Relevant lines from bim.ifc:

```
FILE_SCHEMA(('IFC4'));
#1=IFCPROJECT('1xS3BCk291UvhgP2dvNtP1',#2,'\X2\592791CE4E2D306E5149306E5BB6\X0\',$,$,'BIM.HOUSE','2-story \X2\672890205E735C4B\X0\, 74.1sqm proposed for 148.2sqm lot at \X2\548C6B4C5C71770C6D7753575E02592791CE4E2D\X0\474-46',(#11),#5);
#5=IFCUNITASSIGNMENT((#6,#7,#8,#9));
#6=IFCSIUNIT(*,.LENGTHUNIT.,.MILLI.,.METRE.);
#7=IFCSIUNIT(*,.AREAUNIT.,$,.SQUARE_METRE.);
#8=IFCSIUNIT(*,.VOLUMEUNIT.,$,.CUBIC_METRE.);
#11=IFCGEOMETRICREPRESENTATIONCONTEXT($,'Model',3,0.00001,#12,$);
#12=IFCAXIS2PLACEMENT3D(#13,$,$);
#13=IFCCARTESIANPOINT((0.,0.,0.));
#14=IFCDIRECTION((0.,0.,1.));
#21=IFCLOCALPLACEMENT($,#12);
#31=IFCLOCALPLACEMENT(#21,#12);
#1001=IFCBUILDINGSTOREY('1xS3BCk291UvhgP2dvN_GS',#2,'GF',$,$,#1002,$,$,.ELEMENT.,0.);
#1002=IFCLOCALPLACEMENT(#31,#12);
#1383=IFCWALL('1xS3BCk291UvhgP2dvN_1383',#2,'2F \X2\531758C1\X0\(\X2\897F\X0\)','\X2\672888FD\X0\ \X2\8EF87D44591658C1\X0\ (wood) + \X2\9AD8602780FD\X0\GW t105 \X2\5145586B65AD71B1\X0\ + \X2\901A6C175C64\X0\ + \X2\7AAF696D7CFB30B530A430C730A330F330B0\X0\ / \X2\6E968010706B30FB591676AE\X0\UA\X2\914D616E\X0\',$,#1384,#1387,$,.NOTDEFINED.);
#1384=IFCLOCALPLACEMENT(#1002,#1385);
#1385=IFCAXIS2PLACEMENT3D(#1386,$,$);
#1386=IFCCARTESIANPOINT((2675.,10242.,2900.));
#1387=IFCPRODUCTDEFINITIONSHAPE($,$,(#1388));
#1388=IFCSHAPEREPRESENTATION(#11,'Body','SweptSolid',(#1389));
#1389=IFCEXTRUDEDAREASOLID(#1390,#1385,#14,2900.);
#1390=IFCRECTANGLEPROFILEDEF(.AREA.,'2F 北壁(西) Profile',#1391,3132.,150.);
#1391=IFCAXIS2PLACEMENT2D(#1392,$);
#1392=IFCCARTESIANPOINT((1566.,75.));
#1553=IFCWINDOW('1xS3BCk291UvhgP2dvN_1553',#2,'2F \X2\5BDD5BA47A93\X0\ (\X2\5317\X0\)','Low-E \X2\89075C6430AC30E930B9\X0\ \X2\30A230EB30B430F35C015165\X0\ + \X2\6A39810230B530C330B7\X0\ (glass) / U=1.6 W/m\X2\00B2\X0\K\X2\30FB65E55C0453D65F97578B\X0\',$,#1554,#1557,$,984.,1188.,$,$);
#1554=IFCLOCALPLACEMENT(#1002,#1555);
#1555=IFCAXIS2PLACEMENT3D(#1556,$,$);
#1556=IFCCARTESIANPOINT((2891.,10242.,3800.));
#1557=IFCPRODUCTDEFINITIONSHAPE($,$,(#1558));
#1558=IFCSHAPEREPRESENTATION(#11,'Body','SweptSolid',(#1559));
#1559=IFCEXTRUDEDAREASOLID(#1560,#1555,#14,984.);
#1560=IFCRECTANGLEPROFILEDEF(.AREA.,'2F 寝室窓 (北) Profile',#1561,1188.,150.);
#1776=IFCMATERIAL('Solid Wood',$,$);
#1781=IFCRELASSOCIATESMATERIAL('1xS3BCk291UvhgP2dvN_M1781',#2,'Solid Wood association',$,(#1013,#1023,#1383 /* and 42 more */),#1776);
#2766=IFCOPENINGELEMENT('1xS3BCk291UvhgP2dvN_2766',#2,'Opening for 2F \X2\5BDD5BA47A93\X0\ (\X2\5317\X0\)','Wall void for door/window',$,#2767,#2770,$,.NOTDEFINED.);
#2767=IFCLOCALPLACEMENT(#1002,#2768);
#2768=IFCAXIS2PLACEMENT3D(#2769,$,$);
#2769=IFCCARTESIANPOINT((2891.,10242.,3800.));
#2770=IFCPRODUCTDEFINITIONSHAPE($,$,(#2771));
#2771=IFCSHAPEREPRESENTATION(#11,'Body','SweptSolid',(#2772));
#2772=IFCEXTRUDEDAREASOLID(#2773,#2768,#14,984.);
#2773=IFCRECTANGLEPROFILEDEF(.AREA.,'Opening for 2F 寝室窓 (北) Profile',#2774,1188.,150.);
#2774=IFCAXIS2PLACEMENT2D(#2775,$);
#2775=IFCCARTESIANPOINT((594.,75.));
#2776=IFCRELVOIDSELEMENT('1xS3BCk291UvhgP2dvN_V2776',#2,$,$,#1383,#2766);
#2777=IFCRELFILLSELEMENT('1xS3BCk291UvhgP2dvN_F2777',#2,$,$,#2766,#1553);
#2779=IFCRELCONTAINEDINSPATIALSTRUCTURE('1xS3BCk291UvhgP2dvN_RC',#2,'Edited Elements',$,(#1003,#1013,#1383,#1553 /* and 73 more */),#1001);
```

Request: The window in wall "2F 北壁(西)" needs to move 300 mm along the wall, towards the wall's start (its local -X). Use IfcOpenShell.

```python
import ifcopenshell
import ifcopenshell.api.geometry
import ifcopenshell.util.placement
import ifcopenshell.util.unit

model = ifcopenshell.open("bim.ifc")
unit_scale = ifcopenshell.util.unit.calculate_unit_scale(model)

window = model.by_id(1553)
opening = window.FillsVoids[0].RelatingOpeningElement
wall = opening.VoidsElements[0].RelatingBuildingElement

wall_matrix = ifcopenshell.util.placement.get_local_placement(wall.ObjectPlacement)
shift = wall_matrix[:3, 0] * -0.3 / unit_scale
before = ifcopenshell.util.placement.get_local_placement(window.ObjectPlacement)[:3, 3].copy()

# The window is not placed relative to its opening, so move both.
for product in (opening, window):
    matrix = ifcopenshell.util.placement.get_local_placement(product.ObjectPlacement)
    matrix[:3, 3] += shift
    ifcopenshell.api.geometry.edit_object_placement(model, product=product, matrix=matrix, is_si=False)

after = ifcopenshell.util.placement.get_local_placement(window.ObjectPlacement)[:3, 3]
print("window moved by", (after - before).round(3) + 0.0)

model.write("bim-out.ifc")
```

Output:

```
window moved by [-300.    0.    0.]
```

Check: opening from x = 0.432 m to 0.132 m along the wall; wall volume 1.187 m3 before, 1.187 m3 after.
